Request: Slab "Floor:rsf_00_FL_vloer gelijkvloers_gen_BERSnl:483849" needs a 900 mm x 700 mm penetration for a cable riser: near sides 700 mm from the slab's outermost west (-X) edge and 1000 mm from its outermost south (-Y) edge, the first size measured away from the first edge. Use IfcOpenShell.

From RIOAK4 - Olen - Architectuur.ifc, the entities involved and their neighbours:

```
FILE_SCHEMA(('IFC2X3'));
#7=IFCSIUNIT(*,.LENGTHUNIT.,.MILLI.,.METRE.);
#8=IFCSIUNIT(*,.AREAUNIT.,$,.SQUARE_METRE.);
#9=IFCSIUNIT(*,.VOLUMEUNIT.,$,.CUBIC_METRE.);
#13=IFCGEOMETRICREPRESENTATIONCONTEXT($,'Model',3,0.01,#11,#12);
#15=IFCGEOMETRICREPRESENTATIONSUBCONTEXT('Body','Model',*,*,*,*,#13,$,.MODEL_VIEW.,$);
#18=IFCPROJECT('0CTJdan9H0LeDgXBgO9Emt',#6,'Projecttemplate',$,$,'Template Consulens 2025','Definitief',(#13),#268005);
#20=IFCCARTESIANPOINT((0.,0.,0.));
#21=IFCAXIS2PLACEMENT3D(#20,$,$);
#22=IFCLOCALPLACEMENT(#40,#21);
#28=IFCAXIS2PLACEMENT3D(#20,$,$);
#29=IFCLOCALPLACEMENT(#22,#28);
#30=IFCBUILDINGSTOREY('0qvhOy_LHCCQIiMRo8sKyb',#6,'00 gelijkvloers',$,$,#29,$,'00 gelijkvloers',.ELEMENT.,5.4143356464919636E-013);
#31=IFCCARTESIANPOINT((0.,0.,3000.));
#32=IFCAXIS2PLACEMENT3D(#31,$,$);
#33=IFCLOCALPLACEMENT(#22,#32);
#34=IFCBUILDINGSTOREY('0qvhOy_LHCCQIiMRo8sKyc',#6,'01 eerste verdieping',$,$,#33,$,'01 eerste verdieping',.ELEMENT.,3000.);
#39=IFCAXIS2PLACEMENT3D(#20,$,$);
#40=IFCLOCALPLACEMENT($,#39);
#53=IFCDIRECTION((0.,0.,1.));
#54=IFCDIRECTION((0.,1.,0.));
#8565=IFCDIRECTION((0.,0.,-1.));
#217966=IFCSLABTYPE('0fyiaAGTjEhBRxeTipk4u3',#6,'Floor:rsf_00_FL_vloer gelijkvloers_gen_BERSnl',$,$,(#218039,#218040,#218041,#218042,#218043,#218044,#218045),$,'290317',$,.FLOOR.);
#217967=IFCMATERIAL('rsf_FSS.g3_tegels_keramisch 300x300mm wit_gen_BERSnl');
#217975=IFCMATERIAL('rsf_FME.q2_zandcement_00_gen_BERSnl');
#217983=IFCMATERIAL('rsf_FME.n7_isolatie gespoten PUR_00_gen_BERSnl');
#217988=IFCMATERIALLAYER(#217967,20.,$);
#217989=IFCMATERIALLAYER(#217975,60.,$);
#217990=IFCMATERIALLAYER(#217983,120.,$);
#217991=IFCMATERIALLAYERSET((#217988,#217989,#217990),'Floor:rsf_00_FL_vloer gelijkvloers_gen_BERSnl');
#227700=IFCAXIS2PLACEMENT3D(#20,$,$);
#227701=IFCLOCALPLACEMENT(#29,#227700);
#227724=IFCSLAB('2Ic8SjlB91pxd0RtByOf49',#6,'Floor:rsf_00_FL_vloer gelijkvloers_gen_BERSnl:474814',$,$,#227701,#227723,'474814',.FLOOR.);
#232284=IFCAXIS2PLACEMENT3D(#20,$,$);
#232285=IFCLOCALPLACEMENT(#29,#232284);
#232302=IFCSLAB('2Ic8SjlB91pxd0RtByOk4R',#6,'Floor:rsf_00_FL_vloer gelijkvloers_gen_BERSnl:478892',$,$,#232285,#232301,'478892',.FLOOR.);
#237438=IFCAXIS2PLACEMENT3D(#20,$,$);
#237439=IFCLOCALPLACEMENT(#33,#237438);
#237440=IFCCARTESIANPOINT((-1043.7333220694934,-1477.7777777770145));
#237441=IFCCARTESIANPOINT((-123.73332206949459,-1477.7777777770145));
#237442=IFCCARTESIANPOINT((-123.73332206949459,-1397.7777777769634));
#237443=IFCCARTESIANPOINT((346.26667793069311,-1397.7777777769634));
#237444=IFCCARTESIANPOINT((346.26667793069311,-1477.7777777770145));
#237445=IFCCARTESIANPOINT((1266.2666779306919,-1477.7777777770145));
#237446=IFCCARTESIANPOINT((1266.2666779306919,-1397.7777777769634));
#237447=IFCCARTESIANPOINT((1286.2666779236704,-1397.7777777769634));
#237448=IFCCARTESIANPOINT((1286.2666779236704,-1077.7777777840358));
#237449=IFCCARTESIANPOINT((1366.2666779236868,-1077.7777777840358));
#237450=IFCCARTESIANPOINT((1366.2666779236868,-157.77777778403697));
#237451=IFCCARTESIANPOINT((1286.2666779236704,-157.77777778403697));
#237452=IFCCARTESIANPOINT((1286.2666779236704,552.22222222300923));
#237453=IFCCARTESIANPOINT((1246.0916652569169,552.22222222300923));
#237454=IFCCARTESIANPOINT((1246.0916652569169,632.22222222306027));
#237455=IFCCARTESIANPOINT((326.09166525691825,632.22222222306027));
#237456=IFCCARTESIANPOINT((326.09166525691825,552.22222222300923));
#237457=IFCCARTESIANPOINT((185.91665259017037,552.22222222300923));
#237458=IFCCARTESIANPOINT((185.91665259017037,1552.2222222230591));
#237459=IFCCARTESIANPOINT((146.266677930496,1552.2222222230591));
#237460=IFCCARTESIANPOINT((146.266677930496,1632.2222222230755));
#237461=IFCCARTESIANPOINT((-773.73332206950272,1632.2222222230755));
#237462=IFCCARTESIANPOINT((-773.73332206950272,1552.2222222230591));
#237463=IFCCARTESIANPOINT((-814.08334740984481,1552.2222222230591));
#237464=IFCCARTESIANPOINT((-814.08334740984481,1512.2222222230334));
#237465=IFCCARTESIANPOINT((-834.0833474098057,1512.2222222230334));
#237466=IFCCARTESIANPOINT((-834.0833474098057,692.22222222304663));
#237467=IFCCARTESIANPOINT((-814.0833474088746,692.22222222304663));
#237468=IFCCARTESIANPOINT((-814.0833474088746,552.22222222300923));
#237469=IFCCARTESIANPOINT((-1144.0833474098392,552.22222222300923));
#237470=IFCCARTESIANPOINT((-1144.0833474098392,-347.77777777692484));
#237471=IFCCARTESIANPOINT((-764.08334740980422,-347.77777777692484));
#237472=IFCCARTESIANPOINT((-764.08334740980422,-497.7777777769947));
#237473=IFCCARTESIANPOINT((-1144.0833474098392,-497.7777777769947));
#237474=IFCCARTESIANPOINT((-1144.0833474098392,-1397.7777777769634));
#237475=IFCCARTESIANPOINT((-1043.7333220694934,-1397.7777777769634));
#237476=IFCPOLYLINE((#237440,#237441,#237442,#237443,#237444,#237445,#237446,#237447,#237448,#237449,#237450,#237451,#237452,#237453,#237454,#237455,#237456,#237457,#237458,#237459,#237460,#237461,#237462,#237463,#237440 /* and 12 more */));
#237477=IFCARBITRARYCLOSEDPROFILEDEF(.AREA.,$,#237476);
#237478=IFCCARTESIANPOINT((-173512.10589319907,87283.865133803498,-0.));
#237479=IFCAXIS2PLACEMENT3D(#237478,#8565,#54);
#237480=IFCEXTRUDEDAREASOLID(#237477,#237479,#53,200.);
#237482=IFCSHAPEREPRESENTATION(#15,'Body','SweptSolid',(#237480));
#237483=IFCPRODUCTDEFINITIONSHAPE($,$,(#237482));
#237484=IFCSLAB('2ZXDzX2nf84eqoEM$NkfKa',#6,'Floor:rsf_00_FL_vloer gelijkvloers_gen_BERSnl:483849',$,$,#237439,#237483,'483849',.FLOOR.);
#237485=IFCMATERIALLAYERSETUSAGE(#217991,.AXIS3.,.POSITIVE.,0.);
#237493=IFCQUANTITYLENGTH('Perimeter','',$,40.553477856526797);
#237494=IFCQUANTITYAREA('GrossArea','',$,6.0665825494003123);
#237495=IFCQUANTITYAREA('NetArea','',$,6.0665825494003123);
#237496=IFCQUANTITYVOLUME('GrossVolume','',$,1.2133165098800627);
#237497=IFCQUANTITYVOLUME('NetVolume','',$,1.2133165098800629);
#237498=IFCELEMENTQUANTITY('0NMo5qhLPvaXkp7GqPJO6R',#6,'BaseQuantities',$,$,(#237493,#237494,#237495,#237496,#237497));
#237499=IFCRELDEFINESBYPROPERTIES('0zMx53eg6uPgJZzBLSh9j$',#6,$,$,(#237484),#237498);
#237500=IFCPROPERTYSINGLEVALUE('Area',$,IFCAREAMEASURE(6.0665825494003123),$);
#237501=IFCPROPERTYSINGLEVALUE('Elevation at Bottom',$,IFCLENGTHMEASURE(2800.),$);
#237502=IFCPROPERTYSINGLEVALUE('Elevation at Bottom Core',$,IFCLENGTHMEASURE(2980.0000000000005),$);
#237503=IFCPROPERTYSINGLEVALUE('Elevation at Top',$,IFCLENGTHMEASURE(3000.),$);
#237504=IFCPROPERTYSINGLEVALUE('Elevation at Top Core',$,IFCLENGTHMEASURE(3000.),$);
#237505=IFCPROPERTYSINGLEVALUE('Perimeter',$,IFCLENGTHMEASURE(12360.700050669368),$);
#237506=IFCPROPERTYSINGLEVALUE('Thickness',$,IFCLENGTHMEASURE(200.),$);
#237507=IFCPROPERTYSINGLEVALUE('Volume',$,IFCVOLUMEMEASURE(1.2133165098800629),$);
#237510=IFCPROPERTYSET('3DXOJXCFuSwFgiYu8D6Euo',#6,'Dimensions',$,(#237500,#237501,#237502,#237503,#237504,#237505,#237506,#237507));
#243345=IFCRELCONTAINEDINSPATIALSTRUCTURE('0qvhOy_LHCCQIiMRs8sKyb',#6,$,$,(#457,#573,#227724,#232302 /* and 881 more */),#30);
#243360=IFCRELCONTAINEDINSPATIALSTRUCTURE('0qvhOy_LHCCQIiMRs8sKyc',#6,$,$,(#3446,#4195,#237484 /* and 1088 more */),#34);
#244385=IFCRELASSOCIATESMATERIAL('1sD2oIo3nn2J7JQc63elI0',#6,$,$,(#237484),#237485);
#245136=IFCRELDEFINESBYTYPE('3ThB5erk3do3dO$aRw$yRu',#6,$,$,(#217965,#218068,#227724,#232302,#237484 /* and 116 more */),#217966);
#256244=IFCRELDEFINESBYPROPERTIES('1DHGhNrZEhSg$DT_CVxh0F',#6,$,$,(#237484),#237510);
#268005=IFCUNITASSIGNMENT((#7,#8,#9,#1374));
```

```python
import numpy as np
import ifcopenshell
import ifcopenshell.api.feature
import ifcopenshell.api.geometry
import ifcopenshell.api.pset
import ifcopenshell.api.root
import ifcopenshell.geom
import ifcopenshell.util.element
import ifcopenshell.util.placement
import ifcopenshell.util.representation
import ifcopenshell.util.shape
import ifcopenshell.util.unit

model = ifcopenshell.open("RIOAK4 - Olen - Architectuur.ifc")
unit_scale = ifcopenshell.util.unit.calculate_unit_scale(model)
area_scale = ifcopenshell.util.unit.calculate_unit_scale(model, "AREAUNIT")
volume_scale = ifcopenshell.util.unit.calculate_unit_scale(model, "VOLUMEUNIT")
settings = ifcopenshell.geom.settings()


def volume(element):
    """Net volume in cubic metres, openings subtracted."""
    shape = ifcopenshell.geom.create_shape(settings, element)
    return ifcopenshell.util.shape.get_volume(shape.geometry)


slab = model.by_guid("2ZXDzX2nf84eqoEM$NkfKa")
before = volume(slab)

# Extent in the slab's own axes, in metres. The edges named are its -X and -Y sides.
slab_shape = ifcopenshell.geom.create_shape(settings, slab)
vertices = ifcopenshell.util.shape.get_vertices(slab_shape.geometry)
x_min, y_min, bottom = vertices.min(axis=0)
top = vertices[:, 2].max()

opening = ifcopenshell.api.root.create_entity(model, ifc_class="IfcOpeningElement", name="Cable riser opening")
context = ifcopenshell.util.representation.get_context(model, "Model", "Body", "MODEL_VIEW")
width, depth = 0.9, 0.7
outline = [(0.0, 0.0), (width, 0.0), (width, depth), (0.0, depth), (0.0, 0.0)]
# Overshoot both faces by 50 mm so the cut is clean.
shape = ifcopenshell.api.geometry.add_slab_representation(
    model, context=context, depth=top - bottom + 0.1, polyline=outline
)
ifcopenshell.api.geometry.assign_representation(model, product=opening, representation=shape)

matrix = ifcopenshell.util.placement.get_local_placement(slab.ObjectPlacement)
matrix[:, 3] = matrix @ np.append(np.array([x_min + 0.7, y_min + 1, bottom - 0.05]) / unit_scale, 1.0)
ifcopenshell.api.geometry.edit_object_placement(model, product=opening, matrix=matrix, is_si=False)
ifcopenshell.api.feature.add_feature(model, feature=opening, element=slab)

after = volume(slab)

# Update the slab's stored quantities.
qto = model.by_id(ifcopenshell.util.element.get_pset(slab, "BaseQuantities", should_inherit=False)["id"])
ifcopenshell.api.pset.edit_qto(model, qto=qto, properties={
    "NetArea": after / (top - bottom) / area_scale,
    "NetVolume": after / volume_scale,
})
pset = model.by_id(ifcopenshell.util.element.get_pset(slab, "Dimensions", should_inherit=False)["id"])
ifcopenshell.api.pset.edit_pset(model, pset=pset, properties={
    "Area": model.create_entity("IfcAreaMeasure", after / (top - bottom) / area_scale),
    "Volume": model.create_entity("IfcVolumeMeasure", after / volume_scale),
})

print(f"slab volume {before:.3f} -> {after:.3f} m3")

model.write("RIOAK4 - Olen - Architectuur_updated.ifc")
```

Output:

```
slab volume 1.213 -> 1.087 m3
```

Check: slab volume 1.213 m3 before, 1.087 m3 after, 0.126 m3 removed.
